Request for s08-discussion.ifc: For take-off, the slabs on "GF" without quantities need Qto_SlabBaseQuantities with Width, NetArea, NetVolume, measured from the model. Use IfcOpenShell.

First a look at what the model holds.

```python
import ifcopenshell
import ifcopenshell.util.element
import ifcopenshell.util.unit

model = ifcopenshell.open("s08-discussion.ifc")
print(model.schema)
for unit_type in ("LENGTHUNIT", "AREAUNIT", "VOLUMEUNIT"):
    print(unit_type, ifcopenshell.util.unit.calculate_unit_scale(model, unit_type))
storey = next(s for s in model.by_type("IfcBuildingStorey") if s.Name == "GF")
slabs = [e for e in ifcopenshell.util.element.get_decomposition(storey) if e.is_a("IfcSlab")]
for e in sorted(slabs, key=lambda e: e.id()):
    print(e.id(), e.is_a(), e.Name, list(ifcopenshell.util.element.get_psets(e, qtos_only=True)), sep=" | ")
```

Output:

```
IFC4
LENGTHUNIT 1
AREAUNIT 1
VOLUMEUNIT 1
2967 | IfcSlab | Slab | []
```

```python
import ifcopenshell
import ifcopenshell.api.pset
import ifcopenshell.geom
import ifcopenshell.util.element
import ifcopenshell.util.shape
import ifcopenshell.util.unit

model = ifcopenshell.open("s08-discussion.ifc")
unit_scale = ifcopenshell.util.unit.calculate_unit_scale(model)
area_scale = ifcopenshell.util.unit.calculate_unit_scale(model, "AREAUNIT")
volume_scale = ifcopenshell.util.unit.calculate_unit_scale(model, "VOLUMEUNIT")
settings = ifcopenshell.geom.settings()

storey = next(s for s in model.by_type("IfcBuildingStorey") if s.Name == "GF")
slabs = [e for e in ifcopenshell.util.element.get_decomposition(storey) if e.is_a("IfcSlab")]

for e in sorted(slabs, key=lambda e: e.id()):
    if ifcopenshell.util.element.get_psets(e, qtos_only=True, should_inherit=False):
        continue
    # Geometry comes back in metres, in the element's own axes.
    shape = ifcopenshell.geom.create_shape(settings, e)
    values = {
        "Width": ifcopenshell.util.shape.get_z(shape.geometry) / unit_scale,
        "NetArea": ifcopenshell.util.shape.get_footprint_area(shape.geometry) / area_scale,
        "NetVolume": ifcopenshell.util.shape.get_volume(shape.geometry) / volume_scale,
    }
    qto = ifcopenshell.api.pset.add_qto(model, product=e, name="Qto_SlabBaseQuantities")
    ifcopenshell.api.pset.edit_qto(model, qto=qto, properties=values)
    print(e.id(), {k: round(v, 3) for k, v in values.items()})

model.write("s08-discussion_rev.ifc")
```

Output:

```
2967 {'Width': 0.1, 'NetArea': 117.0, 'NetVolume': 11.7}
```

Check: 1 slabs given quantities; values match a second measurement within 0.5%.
